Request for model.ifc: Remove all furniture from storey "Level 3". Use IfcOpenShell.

First a look at what the model holds.

```python
import ifcopenshell
import ifcopenshell.util.element

model = ifcopenshell.open("model.ifc")
print(model.schema)
storey = next(s for s in model.by_type("IfcBuildingStorey") if s.Name == "Level 3")
furniture = [e for e in ifcopenshell.util.element.get_decomposition(storey) if e.is_a("IfcFurnishingElement")]
seen = {}
for e in furniture:
    element_type = ifcopenshell.util.element.get_type(e)
    name = element_type.Name if element_type not in (None, e) else None
    seen[name] = seen.get(name, 0) + 1
for name, count in sorted(seen.items(), key=str):
    print(count, "x", name)
```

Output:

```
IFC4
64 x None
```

```python
import ifcopenshell
import ifcopenshell.api.root
import ifcopenshell.util.element

model = ifcopenshell.open("model.ifc")

storey = next(s for s in model.by_type("IfcBuildingStorey") if s.Name == "Level 3")
furniture = [e for e in ifcopenshell.util.element.get_decomposition(storey) if e.is_a("IfcFurnishingElement")]

for e in furniture:
    ifcopenshell.api.root.remove_product(model, product=e)
print(len(furniture), "removed")

model.write("model_rev.ifc")
```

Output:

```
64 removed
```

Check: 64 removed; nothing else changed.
